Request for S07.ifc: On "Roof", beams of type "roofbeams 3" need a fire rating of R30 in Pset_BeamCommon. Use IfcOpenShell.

First a look at what the model holds.

```python
import ifcopenshell
import ifcopenshell.util.element

model = ifcopenshell.open("S07.ifc")
print(model.schema)
storey = next(s for s in model.by_type("IfcBuildingStorey") if s.Name == "Roof")
beams = [e for e in ifcopenshell.util.element.get_decomposition(storey) if e.is_a("IfcBeam")]
seen = {}
for e in beams:
    element_type = ifcopenshell.util.element.get_type(e)
    key = (element_type.Name if element_type != e and element_type else None, ifcopenshell.util.element.get_pset(e, "Pset_BeamCommon", "FireRating"))
    seen[key] = seen.get(key, 0) + 1
for (name, value), count in sorted(seen.items(), key=str):
    print(count, "x", name, "|", value)
```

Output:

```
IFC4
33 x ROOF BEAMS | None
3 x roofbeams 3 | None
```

```python
import ifcopenshell
import ifcopenshell.api.pset
import ifcopenshell.util.element

model = ifcopenshell.open("S07.ifc")

storey = next(s for s in model.by_type("IfcBuildingStorey") if s.Name == "Roof")
beams = [e for e in ifcopenshell.util.element.get_decomposition(storey) if e.is_a("IfcBeam")]

count = 0
for e in beams:
    element_type = ifcopenshell.util.element.get_type(e)
    if element_type in (None, e) or element_type.Name != "roofbeams 3":
        continue
    # add_pset returns the element's existing set when there is one.
    pset = ifcopenshell.api.pset.add_pset(model, product=e, name="Pset_BeamCommon")
    ifcopenshell.api.pset.edit_pset(model, pset=pset, properties={"FireRating": "R30"})
    count += 1

print(count, "beams updated")

model.write("S07_updated.ifc")
```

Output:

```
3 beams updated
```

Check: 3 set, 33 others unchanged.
